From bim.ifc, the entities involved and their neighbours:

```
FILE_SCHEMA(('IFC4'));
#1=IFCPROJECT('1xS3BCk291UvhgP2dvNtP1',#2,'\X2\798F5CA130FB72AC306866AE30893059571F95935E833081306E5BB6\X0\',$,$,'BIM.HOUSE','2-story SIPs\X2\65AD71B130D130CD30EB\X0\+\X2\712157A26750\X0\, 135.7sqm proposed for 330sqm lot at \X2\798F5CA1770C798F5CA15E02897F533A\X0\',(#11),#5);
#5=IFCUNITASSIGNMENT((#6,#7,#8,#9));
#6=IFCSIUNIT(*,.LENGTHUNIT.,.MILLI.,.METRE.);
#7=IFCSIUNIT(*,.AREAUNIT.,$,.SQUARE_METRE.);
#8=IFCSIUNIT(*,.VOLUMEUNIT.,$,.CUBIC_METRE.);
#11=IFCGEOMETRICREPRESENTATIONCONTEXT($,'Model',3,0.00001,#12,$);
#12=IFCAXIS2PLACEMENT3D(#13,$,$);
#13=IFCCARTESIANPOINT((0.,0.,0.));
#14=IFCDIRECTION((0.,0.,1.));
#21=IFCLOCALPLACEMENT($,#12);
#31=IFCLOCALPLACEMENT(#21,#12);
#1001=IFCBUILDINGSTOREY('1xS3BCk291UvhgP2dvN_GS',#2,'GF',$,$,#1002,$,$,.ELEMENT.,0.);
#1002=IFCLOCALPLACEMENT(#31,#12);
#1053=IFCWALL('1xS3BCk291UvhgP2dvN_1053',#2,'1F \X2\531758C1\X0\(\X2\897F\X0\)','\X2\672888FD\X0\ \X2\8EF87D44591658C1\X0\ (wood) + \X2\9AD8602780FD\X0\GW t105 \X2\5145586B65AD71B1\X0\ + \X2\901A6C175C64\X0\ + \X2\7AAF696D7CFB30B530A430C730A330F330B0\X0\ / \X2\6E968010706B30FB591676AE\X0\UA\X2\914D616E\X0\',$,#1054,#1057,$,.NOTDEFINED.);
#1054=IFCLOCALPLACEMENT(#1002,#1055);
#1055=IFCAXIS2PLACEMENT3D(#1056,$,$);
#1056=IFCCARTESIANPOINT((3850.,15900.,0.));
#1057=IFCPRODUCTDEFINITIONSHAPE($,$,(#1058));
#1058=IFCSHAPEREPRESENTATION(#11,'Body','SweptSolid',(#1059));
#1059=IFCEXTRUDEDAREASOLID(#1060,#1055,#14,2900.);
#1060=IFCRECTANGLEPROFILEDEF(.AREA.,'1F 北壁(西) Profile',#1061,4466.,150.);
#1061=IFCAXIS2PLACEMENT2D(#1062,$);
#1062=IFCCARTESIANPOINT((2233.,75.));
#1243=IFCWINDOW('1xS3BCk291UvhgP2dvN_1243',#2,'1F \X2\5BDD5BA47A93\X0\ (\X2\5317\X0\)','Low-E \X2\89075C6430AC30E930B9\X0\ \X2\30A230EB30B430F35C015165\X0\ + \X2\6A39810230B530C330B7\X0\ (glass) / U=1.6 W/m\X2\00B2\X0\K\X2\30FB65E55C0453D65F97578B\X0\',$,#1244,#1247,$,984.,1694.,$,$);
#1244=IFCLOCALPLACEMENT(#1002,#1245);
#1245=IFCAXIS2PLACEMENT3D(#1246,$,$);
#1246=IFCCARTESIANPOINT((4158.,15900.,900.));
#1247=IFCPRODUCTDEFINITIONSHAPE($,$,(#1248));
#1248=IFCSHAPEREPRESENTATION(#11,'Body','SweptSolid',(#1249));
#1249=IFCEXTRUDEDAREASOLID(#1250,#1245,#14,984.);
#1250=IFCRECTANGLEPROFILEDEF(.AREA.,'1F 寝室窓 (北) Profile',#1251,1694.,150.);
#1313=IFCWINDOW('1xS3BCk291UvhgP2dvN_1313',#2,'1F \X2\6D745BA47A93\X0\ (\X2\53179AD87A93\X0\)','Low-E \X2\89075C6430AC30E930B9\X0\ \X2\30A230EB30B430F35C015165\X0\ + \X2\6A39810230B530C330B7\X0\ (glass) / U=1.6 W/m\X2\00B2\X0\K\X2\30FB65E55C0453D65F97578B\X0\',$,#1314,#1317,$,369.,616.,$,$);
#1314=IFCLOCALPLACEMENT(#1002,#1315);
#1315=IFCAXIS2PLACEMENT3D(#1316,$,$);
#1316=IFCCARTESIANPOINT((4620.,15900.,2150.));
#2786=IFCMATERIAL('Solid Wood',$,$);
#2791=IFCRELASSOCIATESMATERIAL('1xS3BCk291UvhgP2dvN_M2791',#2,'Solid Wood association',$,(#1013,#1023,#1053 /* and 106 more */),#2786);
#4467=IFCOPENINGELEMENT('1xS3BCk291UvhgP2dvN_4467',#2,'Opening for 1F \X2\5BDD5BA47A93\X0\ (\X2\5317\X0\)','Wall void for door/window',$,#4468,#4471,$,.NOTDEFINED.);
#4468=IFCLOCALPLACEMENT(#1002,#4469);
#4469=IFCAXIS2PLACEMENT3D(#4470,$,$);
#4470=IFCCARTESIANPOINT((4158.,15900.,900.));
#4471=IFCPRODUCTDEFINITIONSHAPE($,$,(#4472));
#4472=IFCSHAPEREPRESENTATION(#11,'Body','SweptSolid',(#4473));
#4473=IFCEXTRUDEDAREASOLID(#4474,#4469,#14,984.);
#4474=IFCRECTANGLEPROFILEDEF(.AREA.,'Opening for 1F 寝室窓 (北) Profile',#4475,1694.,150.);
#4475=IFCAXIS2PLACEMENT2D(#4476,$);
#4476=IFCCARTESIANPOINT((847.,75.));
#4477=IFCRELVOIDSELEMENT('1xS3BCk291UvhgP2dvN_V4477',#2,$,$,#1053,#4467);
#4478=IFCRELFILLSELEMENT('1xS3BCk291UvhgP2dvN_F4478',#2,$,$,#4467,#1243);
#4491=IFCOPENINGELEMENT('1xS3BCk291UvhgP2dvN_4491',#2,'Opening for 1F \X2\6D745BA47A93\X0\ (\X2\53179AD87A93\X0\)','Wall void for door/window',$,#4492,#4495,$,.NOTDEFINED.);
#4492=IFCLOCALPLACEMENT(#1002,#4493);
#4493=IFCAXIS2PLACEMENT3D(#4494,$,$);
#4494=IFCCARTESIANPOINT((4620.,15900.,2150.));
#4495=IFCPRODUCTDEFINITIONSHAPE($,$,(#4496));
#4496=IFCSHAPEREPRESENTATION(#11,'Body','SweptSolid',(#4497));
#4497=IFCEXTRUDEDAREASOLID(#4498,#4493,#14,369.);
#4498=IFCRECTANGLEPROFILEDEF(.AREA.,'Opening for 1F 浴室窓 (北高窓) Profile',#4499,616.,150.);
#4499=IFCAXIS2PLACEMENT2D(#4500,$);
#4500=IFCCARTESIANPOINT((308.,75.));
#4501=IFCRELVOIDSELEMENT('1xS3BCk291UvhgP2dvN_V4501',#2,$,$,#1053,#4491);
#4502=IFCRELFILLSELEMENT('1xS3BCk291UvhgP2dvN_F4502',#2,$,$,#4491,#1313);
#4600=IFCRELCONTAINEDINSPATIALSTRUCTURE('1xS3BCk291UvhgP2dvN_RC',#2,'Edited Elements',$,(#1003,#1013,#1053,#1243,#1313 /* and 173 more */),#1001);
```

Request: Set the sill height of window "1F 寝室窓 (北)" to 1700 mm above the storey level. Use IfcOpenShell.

```python
import numpy as np
import ifcopenshell
import ifcopenshell.api.geometry
import ifcopenshell.geom
import ifcopenshell.util.element
import ifcopenshell.util.placement
import ifcopenshell.util.shape
import ifcopenshell.util.unit

model = ifcopenshell.open("bim.ifc")
unit_scale = ifcopenshell.util.unit.calculate_unit_scale(model)

window = model.by_guid("1xS3BCk291UvhgP2dvN_1243")
opening = window.FillsVoids[0].RelatingOpeningElement
storey = ifcopenshell.util.element.get_container(window, ifc_class="IfcBuildingStorey")
level = ifcopenshell.util.placement.get_local_placement(storey.ObjectPlacement)[2, 3]

# The opening's origin need not be at the sill, so measure its lowest point.
shape = ifcopenshell.geom.create_shape(ifcopenshell.geom.settings(), opening)
bottom = ifcopenshell.util.shape.get_shape_bottom_elevation(shape, shape.geometry) / unit_scale
dz = level + 1700.0 - bottom

shift = np.array([0.0, 0.0, dz])
# The window is not placed relative to its opening, so move both.
for product in (opening, window):
    matrix = ifcopenshell.util.placement.get_local_placement(product.ObjectPlacement)
    matrix[:3, 3] += shift
    ifcopenshell.api.geometry.edit_object_placement(model, product=product, matrix=matrix, is_si=False)

print(f"moved by {dz * unit_scale:+.3f} m")

model.write("bim_v2.ifc")
```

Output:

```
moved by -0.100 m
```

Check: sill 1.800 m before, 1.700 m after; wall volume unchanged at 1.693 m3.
